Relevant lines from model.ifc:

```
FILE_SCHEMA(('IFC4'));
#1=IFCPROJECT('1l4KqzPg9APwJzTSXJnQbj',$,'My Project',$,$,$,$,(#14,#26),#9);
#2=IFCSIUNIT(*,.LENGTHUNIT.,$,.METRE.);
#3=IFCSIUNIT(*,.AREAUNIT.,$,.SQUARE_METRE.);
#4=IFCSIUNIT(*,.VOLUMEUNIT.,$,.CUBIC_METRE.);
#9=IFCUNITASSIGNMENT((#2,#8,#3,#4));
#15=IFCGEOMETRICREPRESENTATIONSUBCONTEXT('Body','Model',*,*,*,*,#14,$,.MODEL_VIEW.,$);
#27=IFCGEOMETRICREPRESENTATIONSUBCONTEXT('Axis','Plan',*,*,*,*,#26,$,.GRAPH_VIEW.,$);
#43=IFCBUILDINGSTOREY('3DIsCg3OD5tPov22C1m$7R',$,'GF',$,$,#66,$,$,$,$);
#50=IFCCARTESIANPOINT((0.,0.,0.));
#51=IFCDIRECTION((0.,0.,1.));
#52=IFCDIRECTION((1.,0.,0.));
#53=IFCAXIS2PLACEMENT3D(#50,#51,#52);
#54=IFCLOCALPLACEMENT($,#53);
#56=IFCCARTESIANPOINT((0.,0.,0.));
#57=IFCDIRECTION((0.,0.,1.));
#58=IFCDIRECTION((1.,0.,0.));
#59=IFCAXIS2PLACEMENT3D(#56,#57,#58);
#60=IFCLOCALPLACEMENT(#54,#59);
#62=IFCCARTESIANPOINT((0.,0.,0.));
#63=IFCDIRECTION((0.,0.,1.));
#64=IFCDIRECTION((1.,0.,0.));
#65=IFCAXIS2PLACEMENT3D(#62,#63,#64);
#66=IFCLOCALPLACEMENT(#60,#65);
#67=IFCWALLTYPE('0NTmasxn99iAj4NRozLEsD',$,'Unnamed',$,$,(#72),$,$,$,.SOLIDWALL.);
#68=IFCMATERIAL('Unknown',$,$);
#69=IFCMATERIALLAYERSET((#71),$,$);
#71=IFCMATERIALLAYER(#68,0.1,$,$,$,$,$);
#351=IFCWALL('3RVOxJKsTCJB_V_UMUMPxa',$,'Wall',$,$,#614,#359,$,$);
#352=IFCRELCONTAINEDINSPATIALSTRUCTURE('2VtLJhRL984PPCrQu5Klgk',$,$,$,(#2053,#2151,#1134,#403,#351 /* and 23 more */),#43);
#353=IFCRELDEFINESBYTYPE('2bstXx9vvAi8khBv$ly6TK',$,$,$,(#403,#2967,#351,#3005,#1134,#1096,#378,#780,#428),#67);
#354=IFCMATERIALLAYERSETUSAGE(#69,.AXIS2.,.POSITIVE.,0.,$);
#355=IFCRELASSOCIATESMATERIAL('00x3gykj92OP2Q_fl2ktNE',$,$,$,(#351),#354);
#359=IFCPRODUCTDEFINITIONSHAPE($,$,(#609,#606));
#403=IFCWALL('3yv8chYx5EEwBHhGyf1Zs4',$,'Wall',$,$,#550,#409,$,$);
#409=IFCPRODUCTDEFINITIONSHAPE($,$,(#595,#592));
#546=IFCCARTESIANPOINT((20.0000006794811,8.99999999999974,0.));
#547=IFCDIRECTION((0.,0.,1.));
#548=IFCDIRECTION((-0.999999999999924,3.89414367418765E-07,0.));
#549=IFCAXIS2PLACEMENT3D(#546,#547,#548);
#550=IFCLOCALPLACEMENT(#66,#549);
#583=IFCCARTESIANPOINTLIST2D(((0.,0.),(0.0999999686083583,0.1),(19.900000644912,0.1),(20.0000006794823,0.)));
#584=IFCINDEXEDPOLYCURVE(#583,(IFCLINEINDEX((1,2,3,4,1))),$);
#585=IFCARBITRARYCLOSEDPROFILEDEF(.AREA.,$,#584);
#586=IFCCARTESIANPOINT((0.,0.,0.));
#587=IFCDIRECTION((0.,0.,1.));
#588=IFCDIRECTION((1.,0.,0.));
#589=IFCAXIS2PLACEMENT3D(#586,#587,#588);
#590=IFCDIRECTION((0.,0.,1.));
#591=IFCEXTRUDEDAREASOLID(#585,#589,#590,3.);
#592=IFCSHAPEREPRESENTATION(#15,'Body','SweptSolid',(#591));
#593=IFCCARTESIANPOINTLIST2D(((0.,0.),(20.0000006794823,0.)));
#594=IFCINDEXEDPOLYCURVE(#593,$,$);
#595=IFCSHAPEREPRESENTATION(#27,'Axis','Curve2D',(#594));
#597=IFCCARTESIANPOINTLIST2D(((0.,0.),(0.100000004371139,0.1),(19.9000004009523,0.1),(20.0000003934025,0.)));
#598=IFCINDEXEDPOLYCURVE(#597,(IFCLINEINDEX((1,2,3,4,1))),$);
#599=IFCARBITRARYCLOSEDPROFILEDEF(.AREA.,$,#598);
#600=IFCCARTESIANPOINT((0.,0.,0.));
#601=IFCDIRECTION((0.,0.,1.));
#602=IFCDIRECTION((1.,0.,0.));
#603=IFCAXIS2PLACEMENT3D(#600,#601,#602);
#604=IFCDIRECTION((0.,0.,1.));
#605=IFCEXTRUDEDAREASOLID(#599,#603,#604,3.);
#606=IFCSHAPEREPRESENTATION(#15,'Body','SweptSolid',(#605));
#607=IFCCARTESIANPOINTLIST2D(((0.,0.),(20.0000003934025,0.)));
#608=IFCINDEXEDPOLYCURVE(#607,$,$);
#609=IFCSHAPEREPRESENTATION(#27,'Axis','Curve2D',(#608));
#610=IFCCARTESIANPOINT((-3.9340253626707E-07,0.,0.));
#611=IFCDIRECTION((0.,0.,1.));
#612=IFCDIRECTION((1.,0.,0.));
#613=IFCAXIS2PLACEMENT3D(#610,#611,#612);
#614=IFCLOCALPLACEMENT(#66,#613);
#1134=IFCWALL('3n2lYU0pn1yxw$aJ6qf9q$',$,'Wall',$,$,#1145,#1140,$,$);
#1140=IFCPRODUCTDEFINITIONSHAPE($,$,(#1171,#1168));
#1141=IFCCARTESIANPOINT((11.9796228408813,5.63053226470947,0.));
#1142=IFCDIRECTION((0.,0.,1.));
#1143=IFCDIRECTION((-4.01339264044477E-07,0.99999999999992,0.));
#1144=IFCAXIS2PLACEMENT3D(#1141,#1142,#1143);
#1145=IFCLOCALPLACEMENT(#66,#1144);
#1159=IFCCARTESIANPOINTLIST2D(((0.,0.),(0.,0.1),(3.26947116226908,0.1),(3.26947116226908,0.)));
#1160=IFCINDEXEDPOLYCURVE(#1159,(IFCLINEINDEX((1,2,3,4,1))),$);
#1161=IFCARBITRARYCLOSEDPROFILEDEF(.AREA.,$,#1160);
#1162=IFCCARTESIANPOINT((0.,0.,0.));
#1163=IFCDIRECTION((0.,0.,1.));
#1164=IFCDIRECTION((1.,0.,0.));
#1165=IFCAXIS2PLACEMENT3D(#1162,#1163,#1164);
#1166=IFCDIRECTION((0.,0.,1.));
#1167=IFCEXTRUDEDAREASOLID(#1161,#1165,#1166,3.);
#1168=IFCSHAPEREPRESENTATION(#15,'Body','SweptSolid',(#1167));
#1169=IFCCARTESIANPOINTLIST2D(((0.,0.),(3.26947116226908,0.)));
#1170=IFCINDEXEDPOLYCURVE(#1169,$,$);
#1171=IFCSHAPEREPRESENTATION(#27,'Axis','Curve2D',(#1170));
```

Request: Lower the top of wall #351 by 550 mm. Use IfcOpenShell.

```python
import ifcopenshell
import ifcopenshell.geom
import ifcopenshell.util.representation
import ifcopenshell.util.shape
import ifcopenshell.util.unit

model = ifcopenshell.open("model.ifc")
unit_scale = ifcopenshell.util.unit.calculate_unit_scale(model)
settings = ifcopenshell.geom.settings()


def volume(element):
    """Net volume in cubic metres, openings subtracted."""
    shape = ifcopenshell.geom.create_shape(settings, element)
    return ifcopenshell.util.shape.get_volume(shape.geometry)


wall = model.by_guid("3RVOxJKsTCJB_V_UMUMPxa")
before = volume(wall)

body = ifcopenshell.util.representation.get_representation(wall, "Model", "Body")
solid = body.Items[0]
old_height = solid.Depth
solid.Depth -= 0.55 / unit_scale
after = volume(wall)

print(f"height {old_height:g} -> {solid.Depth:g}, volume {before:.3f} -> {after:.3f} m3")

model.write("model_v2.ifc")
```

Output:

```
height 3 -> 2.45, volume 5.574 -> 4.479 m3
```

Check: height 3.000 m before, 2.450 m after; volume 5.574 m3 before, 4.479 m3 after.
